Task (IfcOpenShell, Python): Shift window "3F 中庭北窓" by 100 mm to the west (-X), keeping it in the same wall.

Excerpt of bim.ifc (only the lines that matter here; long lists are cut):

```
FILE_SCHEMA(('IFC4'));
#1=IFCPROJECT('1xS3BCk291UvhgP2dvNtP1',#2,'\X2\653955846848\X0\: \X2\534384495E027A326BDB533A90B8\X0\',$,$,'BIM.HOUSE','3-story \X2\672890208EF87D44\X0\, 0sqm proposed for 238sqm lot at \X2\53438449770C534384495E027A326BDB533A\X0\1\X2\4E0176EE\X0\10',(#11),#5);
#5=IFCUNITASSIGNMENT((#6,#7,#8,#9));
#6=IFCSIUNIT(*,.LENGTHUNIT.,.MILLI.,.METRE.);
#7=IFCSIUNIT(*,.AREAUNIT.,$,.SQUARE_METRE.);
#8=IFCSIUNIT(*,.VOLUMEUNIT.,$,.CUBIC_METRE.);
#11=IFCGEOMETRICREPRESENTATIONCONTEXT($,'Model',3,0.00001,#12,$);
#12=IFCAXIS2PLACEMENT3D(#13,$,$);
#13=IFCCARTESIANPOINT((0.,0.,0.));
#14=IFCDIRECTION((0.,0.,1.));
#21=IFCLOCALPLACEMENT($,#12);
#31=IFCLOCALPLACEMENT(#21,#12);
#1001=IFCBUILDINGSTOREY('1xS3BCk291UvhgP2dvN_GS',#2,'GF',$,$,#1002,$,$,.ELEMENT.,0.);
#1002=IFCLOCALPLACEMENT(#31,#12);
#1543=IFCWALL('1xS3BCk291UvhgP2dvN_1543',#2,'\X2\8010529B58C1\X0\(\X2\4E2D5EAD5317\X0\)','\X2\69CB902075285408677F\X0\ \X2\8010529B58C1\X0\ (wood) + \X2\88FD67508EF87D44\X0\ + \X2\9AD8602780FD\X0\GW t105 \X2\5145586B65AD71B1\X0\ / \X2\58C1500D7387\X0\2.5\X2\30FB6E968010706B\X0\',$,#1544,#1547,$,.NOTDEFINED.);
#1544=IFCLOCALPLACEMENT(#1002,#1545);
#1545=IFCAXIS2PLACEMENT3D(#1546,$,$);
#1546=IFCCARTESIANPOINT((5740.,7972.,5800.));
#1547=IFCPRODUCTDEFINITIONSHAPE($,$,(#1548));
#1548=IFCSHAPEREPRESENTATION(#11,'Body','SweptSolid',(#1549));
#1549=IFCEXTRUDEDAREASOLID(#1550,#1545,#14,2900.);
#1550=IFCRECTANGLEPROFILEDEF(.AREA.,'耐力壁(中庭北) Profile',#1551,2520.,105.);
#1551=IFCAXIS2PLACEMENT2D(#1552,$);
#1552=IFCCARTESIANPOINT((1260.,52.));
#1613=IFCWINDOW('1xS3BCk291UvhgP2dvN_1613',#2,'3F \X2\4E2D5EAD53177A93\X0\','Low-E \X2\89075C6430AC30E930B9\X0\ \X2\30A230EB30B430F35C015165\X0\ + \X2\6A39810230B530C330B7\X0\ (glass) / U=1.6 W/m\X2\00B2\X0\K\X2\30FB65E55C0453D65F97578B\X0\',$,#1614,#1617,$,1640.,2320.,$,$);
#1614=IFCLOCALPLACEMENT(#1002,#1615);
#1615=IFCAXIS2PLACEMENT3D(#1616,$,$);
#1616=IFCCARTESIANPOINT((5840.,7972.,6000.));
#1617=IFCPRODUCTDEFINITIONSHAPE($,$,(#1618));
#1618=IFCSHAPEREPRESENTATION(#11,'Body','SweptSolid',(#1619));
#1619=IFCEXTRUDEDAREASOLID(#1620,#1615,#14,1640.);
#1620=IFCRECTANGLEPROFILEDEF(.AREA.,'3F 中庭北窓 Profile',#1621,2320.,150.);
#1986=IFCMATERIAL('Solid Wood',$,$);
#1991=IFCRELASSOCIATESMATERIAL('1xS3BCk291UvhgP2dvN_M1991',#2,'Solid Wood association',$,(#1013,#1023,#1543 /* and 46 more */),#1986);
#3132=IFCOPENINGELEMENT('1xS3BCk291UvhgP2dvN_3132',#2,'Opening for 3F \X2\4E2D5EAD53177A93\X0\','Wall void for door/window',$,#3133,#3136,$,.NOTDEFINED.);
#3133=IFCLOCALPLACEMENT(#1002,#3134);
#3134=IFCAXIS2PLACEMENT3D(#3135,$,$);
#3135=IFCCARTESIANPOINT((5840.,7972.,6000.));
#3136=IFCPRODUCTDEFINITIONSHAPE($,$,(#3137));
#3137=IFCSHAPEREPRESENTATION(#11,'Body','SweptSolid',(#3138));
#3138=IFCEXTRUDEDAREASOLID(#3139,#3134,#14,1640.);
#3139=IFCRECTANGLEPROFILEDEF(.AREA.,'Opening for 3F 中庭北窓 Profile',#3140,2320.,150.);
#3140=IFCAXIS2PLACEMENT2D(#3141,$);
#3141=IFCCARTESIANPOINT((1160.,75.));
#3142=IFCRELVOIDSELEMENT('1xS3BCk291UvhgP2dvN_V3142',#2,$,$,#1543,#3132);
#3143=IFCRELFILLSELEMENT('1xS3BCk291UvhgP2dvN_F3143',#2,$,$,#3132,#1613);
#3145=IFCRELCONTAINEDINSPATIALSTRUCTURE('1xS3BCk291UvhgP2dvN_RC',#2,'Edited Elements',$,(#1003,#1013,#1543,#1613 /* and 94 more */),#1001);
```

```python
import ifcopenshell
import ifcopenshell.api.geometry
import ifcopenshell.util.placement
import ifcopenshell.util.unit

model = ifcopenshell.open("bim.ifc")
unit_scale = ifcopenshell.util.unit.calculate_unit_scale(model)

window = model.by_id(1613)
opening = window.FillsVoids[0].RelatingOpeningElement
wall = opening.VoidsElements[0].RelatingBuildingElement

wall_matrix = ifcopenshell.util.placement.get_local_placement(wall.ObjectPlacement)
shift = wall_matrix[:3, 0] * -0.1 / unit_scale
before = ifcopenshell.util.placement.get_local_placement(window.ObjectPlacement)[:3, 3].copy()

# The window is not placed relative to its opening, so move both.
for product in (opening, window):
    matrix = ifcopenshell.util.placement.get_local_placement(product.ObjectPlacement)
    matrix[:3, 3] += shift
    ifcopenshell.api.geometry.edit_object_placement(model, product=product, matrix=matrix, is_si=False)

after = ifcopenshell.util.placement.get_local_placement(window.ObjectPlacement)[:3, 3]
print("window moved by", (after - before).round(3) + 0.0)

model.write("bim_edited.ifc")
```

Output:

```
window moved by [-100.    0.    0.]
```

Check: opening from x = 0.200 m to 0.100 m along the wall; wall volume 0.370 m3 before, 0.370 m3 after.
